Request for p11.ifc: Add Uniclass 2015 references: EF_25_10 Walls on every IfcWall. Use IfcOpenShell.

First a look at what the model holds.

```python
import ifcopenshell

model = ifcopenshell.open("p11.ifc")
print(model.schema)
print("classifications:", [c.Name for c in model.by_type("IfcClassification")])
for ifc_class in ("IfcDoor", "IfcRoof", "IfcStair", "IfcWall", "IfcWindow"):
    print(ifc_class, len(model.by_type(ifc_class)))
```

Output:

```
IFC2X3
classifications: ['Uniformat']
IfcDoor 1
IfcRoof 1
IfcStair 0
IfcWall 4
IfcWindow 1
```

```python
import ifcopenshell
import ifcopenshell.api.classification

model = ifcopenshell.open("p11.ifc")

# IFC2X3 requires Source and Edition and has no link from the project to the system.
system = model.create_entity("IfcClassification", Source="NBS", Edition="2015", Name="Uniclass 2015")

codes = {
    "IfcWall": ("EF_25_10", "Walls"),
}
for ifc_class, (code, name) in codes.items():
    products = model.by_type(ifc_class)
    ifcopenshell.api.classification.add_reference(
        model, products=products, classification=system, identification=code, name=name
    )
    print(code, len(products))

model.write("p11_rev.ifc")
```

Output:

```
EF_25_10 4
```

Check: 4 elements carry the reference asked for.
